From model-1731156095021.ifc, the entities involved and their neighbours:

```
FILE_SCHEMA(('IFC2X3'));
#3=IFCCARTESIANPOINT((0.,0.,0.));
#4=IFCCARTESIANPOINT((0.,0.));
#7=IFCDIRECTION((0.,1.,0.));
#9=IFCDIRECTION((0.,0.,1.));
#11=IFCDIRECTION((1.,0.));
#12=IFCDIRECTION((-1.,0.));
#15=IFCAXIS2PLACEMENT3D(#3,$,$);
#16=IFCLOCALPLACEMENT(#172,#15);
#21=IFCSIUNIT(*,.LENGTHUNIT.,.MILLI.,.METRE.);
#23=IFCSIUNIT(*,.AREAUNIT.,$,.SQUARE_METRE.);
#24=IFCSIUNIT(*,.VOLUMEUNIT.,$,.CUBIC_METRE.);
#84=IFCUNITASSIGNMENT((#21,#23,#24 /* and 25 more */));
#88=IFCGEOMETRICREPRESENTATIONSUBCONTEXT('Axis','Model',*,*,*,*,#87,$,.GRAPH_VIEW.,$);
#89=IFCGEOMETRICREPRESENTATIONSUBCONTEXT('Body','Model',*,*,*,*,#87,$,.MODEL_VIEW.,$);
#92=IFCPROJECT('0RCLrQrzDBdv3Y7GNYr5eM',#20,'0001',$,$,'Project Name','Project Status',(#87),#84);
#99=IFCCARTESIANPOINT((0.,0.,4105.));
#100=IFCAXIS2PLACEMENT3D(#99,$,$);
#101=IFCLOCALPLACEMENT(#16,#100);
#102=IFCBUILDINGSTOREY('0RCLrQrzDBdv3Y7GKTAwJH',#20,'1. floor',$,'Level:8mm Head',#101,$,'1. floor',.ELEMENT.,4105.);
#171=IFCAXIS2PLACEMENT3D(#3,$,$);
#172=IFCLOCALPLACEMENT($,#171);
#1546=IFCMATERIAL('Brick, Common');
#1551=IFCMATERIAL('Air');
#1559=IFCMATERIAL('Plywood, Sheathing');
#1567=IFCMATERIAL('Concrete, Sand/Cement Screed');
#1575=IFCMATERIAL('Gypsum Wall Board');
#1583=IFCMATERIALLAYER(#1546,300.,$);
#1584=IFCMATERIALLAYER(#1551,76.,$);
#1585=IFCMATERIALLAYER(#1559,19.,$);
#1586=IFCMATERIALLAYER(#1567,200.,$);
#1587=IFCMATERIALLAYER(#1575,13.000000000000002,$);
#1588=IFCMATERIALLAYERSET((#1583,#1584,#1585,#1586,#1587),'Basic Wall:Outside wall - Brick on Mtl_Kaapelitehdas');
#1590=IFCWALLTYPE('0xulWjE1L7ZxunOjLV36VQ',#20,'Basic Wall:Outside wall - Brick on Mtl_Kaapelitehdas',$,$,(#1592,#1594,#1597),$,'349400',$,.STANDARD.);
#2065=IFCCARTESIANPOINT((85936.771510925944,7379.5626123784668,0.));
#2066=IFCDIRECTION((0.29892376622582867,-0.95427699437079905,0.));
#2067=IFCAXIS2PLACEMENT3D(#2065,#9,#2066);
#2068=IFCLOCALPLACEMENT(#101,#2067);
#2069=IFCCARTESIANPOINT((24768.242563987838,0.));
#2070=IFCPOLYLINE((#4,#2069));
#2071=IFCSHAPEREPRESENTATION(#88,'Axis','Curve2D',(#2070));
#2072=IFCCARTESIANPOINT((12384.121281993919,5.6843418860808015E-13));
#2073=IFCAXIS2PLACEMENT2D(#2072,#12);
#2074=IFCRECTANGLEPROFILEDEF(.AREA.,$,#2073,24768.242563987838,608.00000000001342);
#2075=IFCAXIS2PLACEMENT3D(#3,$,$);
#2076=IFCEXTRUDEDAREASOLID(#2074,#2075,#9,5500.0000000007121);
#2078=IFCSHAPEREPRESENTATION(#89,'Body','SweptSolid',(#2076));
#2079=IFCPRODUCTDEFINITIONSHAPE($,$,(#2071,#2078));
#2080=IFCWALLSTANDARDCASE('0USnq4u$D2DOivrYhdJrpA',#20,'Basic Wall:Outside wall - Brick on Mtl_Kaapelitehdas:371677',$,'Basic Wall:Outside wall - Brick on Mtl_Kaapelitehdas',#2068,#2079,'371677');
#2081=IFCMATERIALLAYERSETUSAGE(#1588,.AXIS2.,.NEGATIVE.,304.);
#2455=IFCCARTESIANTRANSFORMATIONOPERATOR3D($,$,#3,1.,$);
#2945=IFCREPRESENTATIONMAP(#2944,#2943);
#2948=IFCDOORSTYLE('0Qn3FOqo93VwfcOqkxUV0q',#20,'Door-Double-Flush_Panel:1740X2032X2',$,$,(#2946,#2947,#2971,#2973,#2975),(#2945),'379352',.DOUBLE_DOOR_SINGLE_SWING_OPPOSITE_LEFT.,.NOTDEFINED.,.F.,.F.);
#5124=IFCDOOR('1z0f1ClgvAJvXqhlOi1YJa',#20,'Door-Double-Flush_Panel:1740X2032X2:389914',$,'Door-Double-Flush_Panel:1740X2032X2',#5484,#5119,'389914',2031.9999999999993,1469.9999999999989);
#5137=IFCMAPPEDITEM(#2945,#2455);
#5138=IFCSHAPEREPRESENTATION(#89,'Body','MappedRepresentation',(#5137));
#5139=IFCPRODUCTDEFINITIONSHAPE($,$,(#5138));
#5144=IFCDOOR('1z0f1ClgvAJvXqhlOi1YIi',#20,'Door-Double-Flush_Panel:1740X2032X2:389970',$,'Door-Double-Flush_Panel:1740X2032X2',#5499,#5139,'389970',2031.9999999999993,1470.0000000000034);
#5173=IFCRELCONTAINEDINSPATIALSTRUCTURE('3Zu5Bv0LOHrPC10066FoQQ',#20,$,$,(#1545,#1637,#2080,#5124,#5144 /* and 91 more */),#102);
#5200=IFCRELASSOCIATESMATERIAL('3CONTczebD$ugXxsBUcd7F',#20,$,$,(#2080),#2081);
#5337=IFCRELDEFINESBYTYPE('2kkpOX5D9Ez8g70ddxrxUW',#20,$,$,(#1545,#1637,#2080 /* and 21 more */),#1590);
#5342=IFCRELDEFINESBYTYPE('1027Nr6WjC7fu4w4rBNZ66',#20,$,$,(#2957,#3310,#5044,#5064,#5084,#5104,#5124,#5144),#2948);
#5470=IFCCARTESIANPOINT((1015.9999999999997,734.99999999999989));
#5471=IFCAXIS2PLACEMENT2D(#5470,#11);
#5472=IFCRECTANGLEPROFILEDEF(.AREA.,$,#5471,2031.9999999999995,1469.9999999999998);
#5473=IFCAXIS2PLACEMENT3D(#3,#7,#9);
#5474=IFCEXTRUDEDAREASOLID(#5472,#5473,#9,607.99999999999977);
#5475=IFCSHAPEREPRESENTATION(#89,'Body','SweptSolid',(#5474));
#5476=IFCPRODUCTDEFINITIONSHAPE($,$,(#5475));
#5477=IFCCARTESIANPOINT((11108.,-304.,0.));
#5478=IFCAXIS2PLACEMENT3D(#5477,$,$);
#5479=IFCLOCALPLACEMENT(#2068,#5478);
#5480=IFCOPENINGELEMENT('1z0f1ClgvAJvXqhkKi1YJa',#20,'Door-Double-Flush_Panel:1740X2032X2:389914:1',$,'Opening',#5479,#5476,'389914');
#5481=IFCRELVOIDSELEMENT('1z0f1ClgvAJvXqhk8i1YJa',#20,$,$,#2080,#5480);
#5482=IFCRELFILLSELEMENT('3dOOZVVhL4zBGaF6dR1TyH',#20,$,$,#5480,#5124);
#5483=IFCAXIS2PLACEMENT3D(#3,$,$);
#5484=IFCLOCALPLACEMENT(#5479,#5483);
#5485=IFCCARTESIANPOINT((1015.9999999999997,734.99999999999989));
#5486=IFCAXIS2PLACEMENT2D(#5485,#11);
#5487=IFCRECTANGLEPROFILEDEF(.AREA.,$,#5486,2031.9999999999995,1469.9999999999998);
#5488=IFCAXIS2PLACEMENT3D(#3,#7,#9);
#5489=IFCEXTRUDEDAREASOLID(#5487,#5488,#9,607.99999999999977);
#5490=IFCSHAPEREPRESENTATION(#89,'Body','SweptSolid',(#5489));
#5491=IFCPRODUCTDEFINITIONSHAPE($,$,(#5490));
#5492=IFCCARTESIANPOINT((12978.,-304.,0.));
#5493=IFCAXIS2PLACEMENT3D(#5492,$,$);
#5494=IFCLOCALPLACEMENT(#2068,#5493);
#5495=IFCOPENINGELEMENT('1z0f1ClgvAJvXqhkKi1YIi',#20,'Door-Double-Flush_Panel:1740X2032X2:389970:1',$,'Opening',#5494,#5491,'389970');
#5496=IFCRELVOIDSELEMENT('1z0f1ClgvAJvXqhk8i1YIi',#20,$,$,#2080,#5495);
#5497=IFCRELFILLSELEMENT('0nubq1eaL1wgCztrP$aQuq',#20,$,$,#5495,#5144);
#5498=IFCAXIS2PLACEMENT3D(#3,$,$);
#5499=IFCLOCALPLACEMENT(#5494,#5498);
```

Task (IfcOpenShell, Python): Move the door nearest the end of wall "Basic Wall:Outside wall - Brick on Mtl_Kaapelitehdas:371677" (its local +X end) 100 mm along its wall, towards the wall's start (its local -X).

```python
import ifcopenshell
import ifcopenshell.api.geometry
import ifcopenshell.util.placement

model = ifcopenshell.open("model-1731156095021.ifc")

door = model.by_guid("1z0f1ClgvAJvXqhlOi1YIi")
opening = door.FillsVoids[0].RelatingOpeningElement
wall = opening.VoidsElements[0].RelatingBuildingElement

wall_matrix = ifcopenshell.util.placement.get_local_placement(wall.ObjectPlacement)
shift = wall_matrix[:3, 0] * -100.0
before = ifcopenshell.util.placement.get_local_placement(door.ObjectPlacement)[:3, 3].copy()

# The door is placed relative to its opening, so it follows when the opening moves.
matrix = ifcopenshell.util.placement.get_local_placement(opening.ObjectPlacement)
matrix[:3, 3] += shift
ifcopenshell.api.geometry.edit_object_placement(
    model, product=opening, matrix=matrix, is_si=False, should_transform_children=True
)

after = ifcopenshell.util.placement.get_local_placement(door.ObjectPlacement)[:3, 3]
print("door moved by", (after - before).round(3) + 0.0)

model.write("model-1731156095021-out.ifc")
```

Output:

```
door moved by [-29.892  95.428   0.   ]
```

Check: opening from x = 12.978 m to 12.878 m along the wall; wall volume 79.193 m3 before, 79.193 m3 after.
